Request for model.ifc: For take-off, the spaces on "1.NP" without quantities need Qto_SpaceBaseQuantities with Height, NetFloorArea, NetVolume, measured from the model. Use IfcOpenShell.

First a look at what the model holds.

```python
import ifcopenshell
import ifcopenshell.util.element
import ifcopenshell.util.unit

model = ifcopenshell.open("model.ifc")
print(model.schema)
for unit_type in ("LENGTHUNIT", "AREAUNIT", "VOLUMEUNIT"):
    print(unit_type, ifcopenshell.util.unit.calculate_unit_scale(model, unit_type))
storey = next(s for s in model.by_type("IfcBuildingStorey") if s.Name == "1.NP")
spaces = [e for e in ifcopenshell.util.element.get_decomposition(storey) if e.is_a("IfcSpace")]
for e in sorted(spaces, key=lambda e: e.id()):
    print(e.id(), e.is_a(), e.Name, list(ifcopenshell.util.element.get_psets(e, qtos_only=True)), sep=" | ")
```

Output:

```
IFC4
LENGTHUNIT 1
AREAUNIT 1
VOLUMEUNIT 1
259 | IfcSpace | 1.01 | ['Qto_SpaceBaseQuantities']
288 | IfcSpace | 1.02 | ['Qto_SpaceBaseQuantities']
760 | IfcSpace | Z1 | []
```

```python
import ifcopenshell
import ifcopenshell.api.pset
import ifcopenshell.geom
import ifcopenshell.util.element
import ifcopenshell.util.shape
import ifcopenshell.util.unit

model = ifcopenshell.open("model.ifc")
unit_scale = ifcopenshell.util.unit.calculate_unit_scale(model)
area_scale = ifcopenshell.util.unit.calculate_unit_scale(model, "AREAUNIT")
volume_scale = ifcopenshell.util.unit.calculate_unit_scale(model, "VOLUMEUNIT")
settings = ifcopenshell.geom.settings()

storey = next(s for s in model.by_type("IfcBuildingStorey") if s.Name == "1.NP")
spaces = [e for e in ifcopenshell.util.element.get_decomposition(storey) if e.is_a("IfcSpace")]

for e in sorted(spaces, key=lambda e: e.id()):
    if ifcopenshell.util.element.get_psets(e, qtos_only=True, should_inherit=False):
        continue
    # Geometry comes back in metres, in the element's own axes.
    shape = ifcopenshell.geom.create_shape(settings, e)
    values = {
        "Height": ifcopenshell.util.shape.get_z(shape.geometry) / unit_scale,
        "NetFloorArea": ifcopenshell.util.shape.get_footprint_area(shape.geometry) / area_scale,
        "NetVolume": ifcopenshell.util.shape.get_volume(shape.geometry) / volume_scale,
    }
    qto = ifcopenshell.api.pset.add_qto(model, product=e, name="Qto_SpaceBaseQuantities")
    ifcopenshell.api.pset.edit_qto(model, qto=qto, properties=values)
    print(e.id(), {k: round(v, 3) for k, v in values.items()})

model.write("model_rev.ifc")
```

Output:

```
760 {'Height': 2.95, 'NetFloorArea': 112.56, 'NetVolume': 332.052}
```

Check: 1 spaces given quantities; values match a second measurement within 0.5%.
